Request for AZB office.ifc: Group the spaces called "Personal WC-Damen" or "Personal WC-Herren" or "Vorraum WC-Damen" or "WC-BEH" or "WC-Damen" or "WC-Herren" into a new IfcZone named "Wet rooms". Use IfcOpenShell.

First a look at what the model holds.

```python
import ifcopenshell

model = ifcopenshell.open("AZB office.ifc")
print(model.schema)
seen = {}
for space in model.by_type("IfcSpace"):
    seen[space.LongName] = seen.get(space.LongName, 0) + 1
for name, count in sorted(seen.items(), key=str):
    print(count, "x", name)
print("zones:", [z.Name for z in model.by_type("IfcZone")][:20])
```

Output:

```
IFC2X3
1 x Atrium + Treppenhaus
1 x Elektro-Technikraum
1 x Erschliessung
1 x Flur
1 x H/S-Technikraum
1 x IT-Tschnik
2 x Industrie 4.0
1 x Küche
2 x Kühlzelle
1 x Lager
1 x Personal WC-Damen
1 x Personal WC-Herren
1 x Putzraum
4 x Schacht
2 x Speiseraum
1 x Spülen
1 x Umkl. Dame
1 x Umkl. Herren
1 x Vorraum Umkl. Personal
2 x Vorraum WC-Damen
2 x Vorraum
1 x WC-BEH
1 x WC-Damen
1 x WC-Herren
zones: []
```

```python
import ifcopenshell
import ifcopenshell.api.group
import ifcopenshell.api.root

model = ifcopenshell.open("AZB office.ifc")

names = {"Personal WC-Damen", "Personal WC-Herren", "Vorraum WC-Damen", "WC-BEH", "WC-Damen", "WC-Herren"}
spaces = [s for s in model.by_type("IfcSpace") if s.LongName in names]

zone = ifcopenshell.api.root.create_entity(model, ifc_class="IfcZone", name="Wet rooms")
ifcopenshell.api.group.assign_group(model, products=spaces, group=zone)
print(len(spaces), "spaces in", zone.Name)

model.write("AZB office_v2.ifc")
```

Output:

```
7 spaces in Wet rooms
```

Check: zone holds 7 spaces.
